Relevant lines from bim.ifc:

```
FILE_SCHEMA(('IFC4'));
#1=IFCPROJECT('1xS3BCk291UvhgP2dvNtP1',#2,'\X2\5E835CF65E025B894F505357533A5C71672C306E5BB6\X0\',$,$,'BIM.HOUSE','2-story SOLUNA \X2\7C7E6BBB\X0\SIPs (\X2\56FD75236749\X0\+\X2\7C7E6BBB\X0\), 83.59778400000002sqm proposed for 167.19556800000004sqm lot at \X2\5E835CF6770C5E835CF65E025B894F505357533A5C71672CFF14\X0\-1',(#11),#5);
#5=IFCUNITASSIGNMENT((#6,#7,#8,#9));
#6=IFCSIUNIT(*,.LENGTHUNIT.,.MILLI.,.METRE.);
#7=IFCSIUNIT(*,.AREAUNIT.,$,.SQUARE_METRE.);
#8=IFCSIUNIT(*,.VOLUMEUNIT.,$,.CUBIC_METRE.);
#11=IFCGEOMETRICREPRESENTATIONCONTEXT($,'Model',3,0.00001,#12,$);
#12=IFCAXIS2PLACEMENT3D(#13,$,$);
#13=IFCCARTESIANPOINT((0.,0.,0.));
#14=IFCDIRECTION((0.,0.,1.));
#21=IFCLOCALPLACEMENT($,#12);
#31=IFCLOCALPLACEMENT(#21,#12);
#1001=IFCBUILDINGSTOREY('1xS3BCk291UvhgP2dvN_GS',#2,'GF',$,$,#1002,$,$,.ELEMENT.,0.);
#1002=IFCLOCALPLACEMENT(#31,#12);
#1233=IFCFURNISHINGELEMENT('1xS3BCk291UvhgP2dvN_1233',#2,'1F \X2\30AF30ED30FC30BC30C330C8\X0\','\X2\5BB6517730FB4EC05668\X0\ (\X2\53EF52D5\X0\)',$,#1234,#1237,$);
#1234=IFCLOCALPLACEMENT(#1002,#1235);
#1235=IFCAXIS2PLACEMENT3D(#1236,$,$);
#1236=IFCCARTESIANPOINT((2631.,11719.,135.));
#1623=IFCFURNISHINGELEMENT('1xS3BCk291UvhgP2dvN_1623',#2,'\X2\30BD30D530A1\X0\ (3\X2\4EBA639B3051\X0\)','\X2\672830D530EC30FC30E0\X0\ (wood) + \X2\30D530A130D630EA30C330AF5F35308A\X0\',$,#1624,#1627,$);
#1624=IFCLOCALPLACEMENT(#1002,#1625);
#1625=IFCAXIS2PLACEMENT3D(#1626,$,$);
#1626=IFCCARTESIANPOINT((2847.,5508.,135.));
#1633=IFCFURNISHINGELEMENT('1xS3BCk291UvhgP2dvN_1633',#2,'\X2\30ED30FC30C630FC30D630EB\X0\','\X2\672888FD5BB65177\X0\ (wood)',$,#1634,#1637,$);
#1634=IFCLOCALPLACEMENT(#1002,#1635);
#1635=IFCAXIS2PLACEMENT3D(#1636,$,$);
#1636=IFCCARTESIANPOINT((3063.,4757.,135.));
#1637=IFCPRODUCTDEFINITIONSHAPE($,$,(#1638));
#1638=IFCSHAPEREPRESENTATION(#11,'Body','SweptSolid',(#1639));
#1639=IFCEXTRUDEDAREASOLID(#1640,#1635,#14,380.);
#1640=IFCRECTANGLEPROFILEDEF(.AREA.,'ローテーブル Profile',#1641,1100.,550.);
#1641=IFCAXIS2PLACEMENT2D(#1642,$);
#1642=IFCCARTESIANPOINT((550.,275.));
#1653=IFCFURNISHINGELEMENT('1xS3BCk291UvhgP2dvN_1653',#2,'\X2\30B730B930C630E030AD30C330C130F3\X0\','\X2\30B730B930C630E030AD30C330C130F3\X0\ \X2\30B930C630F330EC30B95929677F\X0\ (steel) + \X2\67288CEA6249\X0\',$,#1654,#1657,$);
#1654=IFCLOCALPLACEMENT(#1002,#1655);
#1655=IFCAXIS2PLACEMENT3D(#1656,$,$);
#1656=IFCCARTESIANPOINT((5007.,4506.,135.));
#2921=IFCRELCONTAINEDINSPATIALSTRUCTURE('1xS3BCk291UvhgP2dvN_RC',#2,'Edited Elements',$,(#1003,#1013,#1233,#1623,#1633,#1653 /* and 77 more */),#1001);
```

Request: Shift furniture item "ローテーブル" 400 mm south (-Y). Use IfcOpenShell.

```python
import ifcopenshell
import ifcopenshell.api.geometry
import ifcopenshell.util.placement

model = ifcopenshell.open("bim.ifc")

item = model.by_guid("1xS3BCk291UvhgP2dvN_1633")
matrix = ifcopenshell.util.placement.get_local_placement(item.ObjectPlacement)
matrix[1, 3] -= 400.0
ifcopenshell.api.geometry.edit_object_placement(model, product=item, matrix=matrix, is_si=False)

print(ifcopenshell.util.placement.get_local_placement(item.ObjectPlacement).round(3) + 0.0)

model.write("bim_updated.ifc")
```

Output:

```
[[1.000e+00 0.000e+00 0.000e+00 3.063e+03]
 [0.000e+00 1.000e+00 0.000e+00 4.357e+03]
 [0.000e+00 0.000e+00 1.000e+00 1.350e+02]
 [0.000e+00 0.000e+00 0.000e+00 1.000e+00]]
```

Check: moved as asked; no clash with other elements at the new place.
